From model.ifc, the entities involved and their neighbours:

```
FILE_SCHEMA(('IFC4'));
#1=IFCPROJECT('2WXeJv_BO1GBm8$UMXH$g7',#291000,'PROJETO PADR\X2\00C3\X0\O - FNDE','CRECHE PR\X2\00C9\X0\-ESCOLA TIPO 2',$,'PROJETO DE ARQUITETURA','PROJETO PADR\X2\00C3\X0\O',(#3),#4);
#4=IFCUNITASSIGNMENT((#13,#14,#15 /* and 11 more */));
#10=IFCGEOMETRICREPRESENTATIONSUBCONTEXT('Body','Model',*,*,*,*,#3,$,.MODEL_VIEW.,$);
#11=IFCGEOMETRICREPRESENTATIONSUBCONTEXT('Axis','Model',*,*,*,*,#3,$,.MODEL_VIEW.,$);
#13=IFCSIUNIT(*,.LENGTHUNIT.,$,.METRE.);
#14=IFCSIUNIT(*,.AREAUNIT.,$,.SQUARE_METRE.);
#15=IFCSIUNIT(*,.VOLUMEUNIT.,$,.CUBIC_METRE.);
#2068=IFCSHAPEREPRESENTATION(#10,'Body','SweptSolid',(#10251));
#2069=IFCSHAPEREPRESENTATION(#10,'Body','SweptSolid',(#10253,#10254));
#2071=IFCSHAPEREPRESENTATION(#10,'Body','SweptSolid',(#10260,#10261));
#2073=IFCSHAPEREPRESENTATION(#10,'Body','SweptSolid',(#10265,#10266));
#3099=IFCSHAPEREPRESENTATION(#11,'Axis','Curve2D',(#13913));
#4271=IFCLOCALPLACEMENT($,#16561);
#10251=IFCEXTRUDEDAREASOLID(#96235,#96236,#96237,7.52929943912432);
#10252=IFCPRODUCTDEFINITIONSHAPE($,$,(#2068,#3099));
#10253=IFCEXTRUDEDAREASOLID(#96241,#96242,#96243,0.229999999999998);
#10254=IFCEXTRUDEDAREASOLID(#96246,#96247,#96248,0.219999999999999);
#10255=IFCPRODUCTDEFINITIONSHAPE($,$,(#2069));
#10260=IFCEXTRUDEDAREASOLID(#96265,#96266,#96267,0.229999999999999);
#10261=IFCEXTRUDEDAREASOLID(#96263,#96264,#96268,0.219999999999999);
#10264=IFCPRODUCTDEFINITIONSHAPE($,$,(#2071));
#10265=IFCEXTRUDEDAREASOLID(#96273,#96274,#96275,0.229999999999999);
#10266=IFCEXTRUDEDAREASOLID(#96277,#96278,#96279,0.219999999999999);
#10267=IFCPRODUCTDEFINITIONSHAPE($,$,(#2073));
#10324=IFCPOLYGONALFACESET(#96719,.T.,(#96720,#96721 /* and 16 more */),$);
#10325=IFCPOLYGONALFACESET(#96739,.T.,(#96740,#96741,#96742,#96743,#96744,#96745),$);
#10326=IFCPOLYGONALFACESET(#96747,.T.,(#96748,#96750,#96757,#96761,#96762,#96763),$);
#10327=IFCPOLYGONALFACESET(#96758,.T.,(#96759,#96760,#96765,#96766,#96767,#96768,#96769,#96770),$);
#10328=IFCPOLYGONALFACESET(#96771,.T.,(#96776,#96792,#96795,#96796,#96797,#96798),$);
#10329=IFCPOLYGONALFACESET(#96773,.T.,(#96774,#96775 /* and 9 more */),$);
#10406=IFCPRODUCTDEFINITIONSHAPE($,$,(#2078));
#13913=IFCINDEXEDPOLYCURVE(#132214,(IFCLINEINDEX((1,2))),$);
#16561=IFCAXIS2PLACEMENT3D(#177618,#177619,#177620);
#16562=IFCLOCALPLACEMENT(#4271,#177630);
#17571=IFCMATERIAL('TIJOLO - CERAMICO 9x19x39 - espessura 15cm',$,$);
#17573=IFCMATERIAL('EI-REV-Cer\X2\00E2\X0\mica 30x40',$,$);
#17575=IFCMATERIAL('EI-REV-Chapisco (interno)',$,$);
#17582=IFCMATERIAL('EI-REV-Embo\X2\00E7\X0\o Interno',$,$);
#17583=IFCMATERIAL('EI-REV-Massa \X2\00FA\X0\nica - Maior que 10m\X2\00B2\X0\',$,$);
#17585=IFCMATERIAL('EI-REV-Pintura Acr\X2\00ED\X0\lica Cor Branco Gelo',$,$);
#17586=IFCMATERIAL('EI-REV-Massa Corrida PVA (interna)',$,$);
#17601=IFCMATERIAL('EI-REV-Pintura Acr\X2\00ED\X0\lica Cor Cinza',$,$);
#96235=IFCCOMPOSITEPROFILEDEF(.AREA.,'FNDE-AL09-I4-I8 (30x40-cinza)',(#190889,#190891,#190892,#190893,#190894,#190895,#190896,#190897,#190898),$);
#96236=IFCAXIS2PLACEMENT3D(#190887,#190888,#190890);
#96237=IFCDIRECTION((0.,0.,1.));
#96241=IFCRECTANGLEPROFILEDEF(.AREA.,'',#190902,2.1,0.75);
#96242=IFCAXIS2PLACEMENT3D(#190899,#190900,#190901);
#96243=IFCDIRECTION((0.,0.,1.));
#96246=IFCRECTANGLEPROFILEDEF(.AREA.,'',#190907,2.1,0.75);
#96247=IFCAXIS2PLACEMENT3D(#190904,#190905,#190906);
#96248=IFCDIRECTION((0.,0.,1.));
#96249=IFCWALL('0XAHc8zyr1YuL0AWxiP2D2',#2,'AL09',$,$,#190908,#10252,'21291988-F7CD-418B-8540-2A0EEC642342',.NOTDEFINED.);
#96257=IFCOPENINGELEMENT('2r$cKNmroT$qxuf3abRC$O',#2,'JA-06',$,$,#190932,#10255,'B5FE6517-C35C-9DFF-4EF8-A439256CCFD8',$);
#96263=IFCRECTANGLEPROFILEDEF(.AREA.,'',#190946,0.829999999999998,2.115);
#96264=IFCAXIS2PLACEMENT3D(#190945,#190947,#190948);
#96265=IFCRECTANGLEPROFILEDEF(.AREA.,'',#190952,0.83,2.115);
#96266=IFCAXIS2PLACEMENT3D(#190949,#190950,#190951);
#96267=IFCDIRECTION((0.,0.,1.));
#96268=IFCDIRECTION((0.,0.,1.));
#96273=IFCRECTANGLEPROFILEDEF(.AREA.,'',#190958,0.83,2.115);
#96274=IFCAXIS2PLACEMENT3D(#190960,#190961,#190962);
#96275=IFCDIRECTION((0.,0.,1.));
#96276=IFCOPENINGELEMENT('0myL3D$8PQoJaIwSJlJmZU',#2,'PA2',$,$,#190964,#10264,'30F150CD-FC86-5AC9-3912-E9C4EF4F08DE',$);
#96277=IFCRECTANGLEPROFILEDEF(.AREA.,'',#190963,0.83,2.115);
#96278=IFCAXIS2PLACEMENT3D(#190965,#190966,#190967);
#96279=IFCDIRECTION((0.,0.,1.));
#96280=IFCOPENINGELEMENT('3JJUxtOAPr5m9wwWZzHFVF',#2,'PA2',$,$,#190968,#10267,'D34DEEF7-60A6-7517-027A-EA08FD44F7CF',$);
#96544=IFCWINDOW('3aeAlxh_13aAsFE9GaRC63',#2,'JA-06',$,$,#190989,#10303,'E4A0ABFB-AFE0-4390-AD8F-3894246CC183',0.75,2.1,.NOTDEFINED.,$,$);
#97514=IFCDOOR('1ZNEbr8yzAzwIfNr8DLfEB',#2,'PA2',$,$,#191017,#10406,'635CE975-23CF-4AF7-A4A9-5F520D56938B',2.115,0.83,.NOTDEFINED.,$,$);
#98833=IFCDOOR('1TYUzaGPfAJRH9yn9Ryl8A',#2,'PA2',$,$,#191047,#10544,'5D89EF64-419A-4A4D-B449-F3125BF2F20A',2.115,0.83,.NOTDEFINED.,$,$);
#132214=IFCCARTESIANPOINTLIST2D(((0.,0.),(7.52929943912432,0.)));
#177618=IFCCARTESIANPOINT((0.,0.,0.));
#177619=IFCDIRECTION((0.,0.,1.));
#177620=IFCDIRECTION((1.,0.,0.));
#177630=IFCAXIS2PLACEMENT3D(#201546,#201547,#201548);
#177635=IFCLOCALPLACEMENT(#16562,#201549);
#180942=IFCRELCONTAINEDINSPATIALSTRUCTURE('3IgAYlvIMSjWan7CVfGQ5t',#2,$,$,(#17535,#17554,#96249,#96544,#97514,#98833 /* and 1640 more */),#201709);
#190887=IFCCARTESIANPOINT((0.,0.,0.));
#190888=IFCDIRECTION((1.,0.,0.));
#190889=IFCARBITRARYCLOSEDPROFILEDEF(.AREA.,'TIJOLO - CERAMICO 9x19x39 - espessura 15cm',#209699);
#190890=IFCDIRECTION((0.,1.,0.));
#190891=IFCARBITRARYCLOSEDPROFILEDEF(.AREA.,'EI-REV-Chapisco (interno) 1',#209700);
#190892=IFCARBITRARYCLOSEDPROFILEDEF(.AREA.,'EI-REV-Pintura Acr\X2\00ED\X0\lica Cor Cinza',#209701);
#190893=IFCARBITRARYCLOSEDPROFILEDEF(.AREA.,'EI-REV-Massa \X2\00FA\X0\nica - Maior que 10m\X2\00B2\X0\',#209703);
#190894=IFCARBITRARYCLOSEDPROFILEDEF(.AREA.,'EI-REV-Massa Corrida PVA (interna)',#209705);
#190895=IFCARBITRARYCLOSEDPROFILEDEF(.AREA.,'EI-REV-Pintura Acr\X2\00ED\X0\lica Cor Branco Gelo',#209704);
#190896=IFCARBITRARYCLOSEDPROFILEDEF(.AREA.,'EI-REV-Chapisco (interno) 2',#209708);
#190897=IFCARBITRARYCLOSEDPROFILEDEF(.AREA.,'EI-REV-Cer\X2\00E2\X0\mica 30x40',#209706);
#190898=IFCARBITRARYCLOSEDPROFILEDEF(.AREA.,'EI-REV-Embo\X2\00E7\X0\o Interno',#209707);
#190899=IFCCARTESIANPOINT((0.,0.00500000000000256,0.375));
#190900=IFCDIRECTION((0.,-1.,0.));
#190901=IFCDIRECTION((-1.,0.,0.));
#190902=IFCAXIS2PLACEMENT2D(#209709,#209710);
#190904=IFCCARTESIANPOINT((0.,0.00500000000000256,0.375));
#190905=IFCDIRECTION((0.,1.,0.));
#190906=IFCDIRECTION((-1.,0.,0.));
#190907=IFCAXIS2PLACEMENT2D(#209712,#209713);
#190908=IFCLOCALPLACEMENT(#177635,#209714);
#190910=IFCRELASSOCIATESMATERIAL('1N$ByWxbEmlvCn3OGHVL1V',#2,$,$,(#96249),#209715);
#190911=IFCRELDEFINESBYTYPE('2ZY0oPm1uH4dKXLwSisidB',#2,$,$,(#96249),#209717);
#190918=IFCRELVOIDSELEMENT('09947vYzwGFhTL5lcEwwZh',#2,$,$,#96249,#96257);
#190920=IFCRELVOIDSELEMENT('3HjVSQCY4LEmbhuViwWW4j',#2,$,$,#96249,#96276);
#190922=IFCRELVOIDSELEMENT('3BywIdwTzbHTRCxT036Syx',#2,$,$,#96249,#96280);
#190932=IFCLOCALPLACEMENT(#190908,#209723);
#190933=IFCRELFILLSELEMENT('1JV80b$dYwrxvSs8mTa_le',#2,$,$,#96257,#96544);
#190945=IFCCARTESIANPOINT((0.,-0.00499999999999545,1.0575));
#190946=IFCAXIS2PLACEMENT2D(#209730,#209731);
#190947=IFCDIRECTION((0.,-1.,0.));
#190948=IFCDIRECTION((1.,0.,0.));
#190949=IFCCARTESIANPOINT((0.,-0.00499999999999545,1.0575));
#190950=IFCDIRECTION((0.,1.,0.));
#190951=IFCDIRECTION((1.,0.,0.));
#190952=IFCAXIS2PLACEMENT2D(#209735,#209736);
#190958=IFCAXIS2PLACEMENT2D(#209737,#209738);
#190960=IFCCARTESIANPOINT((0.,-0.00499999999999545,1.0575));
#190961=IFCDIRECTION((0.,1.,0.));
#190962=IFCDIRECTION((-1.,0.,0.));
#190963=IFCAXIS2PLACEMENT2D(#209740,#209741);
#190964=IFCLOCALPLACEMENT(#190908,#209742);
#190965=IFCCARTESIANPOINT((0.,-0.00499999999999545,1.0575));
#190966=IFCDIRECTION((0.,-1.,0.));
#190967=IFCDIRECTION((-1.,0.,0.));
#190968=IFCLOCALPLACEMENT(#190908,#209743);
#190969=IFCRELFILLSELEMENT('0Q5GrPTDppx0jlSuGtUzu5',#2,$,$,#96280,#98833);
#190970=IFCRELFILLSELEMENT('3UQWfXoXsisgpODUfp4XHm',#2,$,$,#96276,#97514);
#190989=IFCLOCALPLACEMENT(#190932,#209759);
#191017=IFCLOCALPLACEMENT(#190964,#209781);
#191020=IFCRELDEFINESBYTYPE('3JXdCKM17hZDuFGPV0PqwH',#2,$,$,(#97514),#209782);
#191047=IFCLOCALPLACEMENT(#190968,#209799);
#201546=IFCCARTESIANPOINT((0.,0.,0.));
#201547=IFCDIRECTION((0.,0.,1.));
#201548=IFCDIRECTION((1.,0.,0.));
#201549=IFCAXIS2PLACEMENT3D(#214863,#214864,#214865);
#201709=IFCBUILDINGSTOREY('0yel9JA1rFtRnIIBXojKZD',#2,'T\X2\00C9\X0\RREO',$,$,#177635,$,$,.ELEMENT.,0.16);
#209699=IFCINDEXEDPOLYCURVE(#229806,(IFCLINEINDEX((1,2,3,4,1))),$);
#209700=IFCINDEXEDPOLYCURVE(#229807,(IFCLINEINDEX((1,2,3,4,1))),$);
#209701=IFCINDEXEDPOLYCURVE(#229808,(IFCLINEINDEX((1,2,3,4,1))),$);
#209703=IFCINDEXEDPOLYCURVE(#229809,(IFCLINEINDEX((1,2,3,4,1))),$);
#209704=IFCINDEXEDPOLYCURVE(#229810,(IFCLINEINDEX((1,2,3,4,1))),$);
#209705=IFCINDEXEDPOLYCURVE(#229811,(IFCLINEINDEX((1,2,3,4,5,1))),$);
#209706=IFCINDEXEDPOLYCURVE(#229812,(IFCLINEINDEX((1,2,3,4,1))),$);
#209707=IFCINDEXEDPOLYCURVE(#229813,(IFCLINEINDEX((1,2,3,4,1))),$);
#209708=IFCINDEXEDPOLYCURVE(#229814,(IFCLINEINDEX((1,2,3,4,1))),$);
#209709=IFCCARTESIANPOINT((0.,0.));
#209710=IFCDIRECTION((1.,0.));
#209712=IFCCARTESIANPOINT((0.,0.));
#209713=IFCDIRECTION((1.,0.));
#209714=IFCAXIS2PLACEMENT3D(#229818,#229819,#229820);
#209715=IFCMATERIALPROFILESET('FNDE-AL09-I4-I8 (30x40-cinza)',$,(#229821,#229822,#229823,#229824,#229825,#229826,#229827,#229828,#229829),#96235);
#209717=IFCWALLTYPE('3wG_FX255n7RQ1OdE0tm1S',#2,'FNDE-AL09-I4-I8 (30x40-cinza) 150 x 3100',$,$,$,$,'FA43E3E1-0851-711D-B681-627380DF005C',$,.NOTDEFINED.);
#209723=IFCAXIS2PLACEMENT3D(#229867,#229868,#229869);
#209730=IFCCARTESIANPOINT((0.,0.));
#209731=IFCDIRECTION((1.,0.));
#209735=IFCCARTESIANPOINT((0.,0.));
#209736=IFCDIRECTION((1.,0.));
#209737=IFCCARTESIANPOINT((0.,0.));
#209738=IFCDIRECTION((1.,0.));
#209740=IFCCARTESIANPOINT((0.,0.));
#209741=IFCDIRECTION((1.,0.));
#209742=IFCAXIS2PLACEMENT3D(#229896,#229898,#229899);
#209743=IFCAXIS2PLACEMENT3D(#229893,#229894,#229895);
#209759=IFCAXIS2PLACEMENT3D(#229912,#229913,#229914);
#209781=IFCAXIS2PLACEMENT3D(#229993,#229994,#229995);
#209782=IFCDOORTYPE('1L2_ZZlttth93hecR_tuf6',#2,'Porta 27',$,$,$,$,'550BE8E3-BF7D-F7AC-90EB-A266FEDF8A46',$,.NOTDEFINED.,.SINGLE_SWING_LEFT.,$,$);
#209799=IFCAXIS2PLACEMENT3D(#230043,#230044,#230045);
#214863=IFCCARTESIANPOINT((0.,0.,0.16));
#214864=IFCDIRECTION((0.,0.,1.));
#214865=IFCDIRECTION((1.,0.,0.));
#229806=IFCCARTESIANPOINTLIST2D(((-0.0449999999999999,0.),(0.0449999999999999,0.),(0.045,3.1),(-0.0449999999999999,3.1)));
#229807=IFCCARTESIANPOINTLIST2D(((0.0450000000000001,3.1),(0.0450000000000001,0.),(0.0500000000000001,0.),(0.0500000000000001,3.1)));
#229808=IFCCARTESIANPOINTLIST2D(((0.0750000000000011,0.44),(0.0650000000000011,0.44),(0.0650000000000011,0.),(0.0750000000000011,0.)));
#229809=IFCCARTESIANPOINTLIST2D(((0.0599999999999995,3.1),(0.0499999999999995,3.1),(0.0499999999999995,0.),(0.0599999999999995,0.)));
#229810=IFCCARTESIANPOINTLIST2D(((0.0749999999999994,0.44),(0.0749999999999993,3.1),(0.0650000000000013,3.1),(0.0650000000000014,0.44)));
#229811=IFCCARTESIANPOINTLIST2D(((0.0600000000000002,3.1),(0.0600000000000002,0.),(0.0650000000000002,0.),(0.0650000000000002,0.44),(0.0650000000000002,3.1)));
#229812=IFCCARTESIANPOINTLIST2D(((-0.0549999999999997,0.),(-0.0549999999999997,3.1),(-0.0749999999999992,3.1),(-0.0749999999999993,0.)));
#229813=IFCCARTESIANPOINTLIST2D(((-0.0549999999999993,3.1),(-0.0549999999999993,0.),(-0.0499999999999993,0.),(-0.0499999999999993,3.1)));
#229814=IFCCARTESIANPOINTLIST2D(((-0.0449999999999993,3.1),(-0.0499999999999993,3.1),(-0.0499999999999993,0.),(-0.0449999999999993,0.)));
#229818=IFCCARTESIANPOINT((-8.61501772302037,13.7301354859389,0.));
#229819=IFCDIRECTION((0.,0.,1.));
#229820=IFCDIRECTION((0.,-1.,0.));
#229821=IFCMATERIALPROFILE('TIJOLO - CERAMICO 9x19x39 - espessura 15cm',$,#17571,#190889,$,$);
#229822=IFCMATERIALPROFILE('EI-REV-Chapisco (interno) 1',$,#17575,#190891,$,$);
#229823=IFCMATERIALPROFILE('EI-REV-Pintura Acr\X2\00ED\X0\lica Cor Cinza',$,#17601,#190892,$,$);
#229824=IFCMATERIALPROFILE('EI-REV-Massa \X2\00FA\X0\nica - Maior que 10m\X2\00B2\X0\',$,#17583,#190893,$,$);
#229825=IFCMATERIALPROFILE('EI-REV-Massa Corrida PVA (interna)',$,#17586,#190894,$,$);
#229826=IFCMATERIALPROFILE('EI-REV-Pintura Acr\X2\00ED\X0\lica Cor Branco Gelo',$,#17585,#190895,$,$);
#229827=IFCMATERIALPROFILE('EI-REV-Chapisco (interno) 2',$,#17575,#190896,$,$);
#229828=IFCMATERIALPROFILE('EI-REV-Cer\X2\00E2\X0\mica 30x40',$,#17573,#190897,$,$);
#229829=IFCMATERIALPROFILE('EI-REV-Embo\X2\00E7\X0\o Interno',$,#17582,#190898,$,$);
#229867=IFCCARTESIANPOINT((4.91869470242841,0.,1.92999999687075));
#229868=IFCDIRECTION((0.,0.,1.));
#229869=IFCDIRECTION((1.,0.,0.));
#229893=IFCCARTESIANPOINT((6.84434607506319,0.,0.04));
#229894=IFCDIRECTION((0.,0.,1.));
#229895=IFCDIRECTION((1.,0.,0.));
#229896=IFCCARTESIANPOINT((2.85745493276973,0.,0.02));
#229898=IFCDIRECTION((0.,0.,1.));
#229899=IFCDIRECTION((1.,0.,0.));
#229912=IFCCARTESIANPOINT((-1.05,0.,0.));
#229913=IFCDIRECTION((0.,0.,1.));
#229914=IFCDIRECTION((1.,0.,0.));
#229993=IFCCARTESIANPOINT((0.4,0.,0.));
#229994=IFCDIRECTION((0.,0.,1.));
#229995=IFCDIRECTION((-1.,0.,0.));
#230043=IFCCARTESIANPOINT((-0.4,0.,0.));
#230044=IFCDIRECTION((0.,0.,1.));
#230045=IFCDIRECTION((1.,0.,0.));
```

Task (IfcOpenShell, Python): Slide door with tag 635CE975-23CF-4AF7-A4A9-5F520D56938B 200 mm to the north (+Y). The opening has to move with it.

```python
import ifcopenshell
import ifcopenshell.api.geometry
import ifcopenshell.util.placement
import ifcopenshell.util.unit

model = ifcopenshell.open("model.ifc")
unit_scale = ifcopenshell.util.unit.calculate_unit_scale(model)

door = model.by_guid("1ZNEbr8yzAzwIfNr8DLfEB")
opening = door.FillsVoids[0].RelatingOpeningElement
wall = opening.VoidsElements[0].RelatingBuildingElement

wall_matrix = ifcopenshell.util.placement.get_local_placement(wall.ObjectPlacement)
shift = wall_matrix[:3, 0] * -0.2 / unit_scale
before = ifcopenshell.util.placement.get_local_placement(door.ObjectPlacement)[:3, 3].copy()

# The door is placed relative to its opening, so it follows when the opening moves.
matrix = ifcopenshell.util.placement.get_local_placement(opening.ObjectPlacement)
matrix[:3, 3] += shift
ifcopenshell.api.geometry.edit_object_placement(
    model, product=opening, matrix=matrix, is_si=False, should_transform_children=True
)

after = ifcopenshell.util.placement.get_local_placement(door.ObjectPlacement)[:3, 3]
print("door moved by", (after - before).round(3) + 0.0)

model.write("model_v2.ifc")
```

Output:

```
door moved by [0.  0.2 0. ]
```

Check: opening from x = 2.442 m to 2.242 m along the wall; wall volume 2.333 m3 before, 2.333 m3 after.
